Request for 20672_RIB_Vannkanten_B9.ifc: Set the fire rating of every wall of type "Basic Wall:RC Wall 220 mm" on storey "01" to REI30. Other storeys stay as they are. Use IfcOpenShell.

First a look at what the model holds.

```python
import ifcopenshell
import ifcopenshell.util.element

model = ifcopenshell.open("20672_RIB_Vannkanten_B9.ifc")
print(model.schema)
storey = next(s for s in model.by_type("IfcBuildingStorey") if s.Name == "01")
walls = [e for e in ifcopenshell.util.element.get_decomposition(storey) if e.is_a("IfcWall")]
seen = {}
for e in walls:
    element_type = ifcopenshell.util.element.get_type(e)
    key = (element_type.Name if element_type != e and element_type else None, ifcopenshell.util.element.get_pset(e, "Pset_WallCommon", "FireRating"))
    seen[key] = seen.get(key, 0) + 1
for (name, value), count in sorted(seen.items(), key=str):
    print(count, "x", name, "|", value)
```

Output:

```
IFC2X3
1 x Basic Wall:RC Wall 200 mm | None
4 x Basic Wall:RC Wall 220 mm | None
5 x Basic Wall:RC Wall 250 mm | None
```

```python
import ifcopenshell
import ifcopenshell.api.pset
import ifcopenshell.util.element

model = ifcopenshell.open("20672_RIB_Vannkanten_B9.ifc")

storey = next(s for s in model.by_type("IfcBuildingStorey") if s.Name == "01")
walls = [e for e in ifcopenshell.util.element.get_decomposition(storey) if e.is_a("IfcWall")]

count = 0
for e in walls:
    element_type = ifcopenshell.util.element.get_type(e)
    if element_type in (None, e) or element_type.Name != "Basic Wall:RC Wall 220 mm":
        continue
    # add_pset returns the element's existing set when there is one.
    pset = ifcopenshell.api.pset.add_pset(model, product=e, name="Pset_WallCommon")
    ifcopenshell.api.pset.edit_pset(model, pset=pset, properties={"FireRating": "REI30"})
    count += 1

print(count, "walls updated")

model.write("20672_RIB_Vannkanten_B9-out.ifc")
```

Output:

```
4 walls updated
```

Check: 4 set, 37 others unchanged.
